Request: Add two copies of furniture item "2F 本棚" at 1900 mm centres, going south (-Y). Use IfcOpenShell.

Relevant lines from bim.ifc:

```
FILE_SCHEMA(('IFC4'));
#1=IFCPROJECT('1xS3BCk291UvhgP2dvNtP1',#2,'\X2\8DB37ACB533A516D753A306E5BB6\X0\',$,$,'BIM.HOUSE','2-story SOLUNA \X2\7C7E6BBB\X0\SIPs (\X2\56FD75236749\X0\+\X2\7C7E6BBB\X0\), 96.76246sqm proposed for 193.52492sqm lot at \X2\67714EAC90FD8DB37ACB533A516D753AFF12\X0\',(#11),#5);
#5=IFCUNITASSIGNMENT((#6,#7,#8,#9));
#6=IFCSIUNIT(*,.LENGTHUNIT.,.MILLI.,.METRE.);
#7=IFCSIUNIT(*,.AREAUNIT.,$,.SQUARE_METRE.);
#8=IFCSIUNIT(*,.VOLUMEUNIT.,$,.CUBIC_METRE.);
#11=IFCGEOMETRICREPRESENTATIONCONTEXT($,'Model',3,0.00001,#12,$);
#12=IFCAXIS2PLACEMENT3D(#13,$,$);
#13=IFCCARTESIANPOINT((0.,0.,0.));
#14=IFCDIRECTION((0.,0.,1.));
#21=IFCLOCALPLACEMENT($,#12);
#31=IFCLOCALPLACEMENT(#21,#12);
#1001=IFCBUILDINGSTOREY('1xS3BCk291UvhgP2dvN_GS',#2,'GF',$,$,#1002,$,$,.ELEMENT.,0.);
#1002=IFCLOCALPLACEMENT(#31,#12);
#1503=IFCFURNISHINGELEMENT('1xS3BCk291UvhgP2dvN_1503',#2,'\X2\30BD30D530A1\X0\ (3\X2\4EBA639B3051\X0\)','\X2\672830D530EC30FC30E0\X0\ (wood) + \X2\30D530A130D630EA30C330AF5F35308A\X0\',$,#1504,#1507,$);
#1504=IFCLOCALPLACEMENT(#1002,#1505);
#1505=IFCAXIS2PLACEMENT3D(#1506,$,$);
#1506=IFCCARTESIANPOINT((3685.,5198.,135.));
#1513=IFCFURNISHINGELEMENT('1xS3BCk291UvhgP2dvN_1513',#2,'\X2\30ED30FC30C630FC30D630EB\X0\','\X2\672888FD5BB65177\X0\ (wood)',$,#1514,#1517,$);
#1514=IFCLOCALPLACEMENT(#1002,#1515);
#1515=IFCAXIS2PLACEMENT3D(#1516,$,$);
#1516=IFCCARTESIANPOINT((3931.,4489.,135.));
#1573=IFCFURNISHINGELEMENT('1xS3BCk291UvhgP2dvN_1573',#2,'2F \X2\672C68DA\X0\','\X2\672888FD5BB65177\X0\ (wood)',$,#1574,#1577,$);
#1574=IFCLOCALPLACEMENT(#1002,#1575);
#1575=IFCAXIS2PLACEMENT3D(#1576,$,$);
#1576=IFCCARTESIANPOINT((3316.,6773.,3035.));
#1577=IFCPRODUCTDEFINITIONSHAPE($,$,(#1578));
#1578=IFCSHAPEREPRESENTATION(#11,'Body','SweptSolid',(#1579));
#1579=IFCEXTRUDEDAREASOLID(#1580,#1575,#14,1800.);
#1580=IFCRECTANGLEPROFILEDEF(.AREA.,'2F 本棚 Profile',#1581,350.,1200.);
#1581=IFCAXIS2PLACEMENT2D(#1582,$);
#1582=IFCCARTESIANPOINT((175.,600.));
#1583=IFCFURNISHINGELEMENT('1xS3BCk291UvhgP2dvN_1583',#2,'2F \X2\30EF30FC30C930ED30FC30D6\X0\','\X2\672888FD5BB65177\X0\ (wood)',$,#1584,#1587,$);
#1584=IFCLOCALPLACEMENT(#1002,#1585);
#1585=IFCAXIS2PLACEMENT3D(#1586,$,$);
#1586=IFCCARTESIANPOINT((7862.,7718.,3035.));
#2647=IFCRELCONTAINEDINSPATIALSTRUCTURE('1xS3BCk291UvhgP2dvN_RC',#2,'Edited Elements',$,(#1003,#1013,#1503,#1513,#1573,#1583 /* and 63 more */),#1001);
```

```python
import numpy as np
import ifcopenshell
import ifcopenshell.api.geometry
import ifcopenshell.api.root
import ifcopenshell.util.element
import ifcopenshell.util.placement

model = ifcopenshell.open("bim.ifc")


def reuse_history(source, copy):
    """copy_class also copies each property set's owner history, people and application; keep the originals."""
    for rel in copy.IsDefinedBy:
        if rel.is_a("IfcRelDefinesByProperties") and (history := rel.RelatingPropertyDefinition.OwnerHistory):
            rel.RelatingPropertyDefinition.OwnerHistory = source.OwnerHistory
            ifcopenshell.util.element.remove_deep2(model, history)


source = model.by_guid("1xS3BCk291UvhgP2dvN_1573")
base = ifcopenshell.util.placement.get_local_placement(source.ObjectPlacement)
step = np.array([0.0, -1.0, 0.0]) * 1900.0

for i in range(1, 3):
    copy = ifcopenshell.api.root.copy_class(model, product=source)
    copy.Representation = ifcopenshell.util.element.copy_deep(
        model, source.Representation, exclude=["IfcGeometricRepresentationContext", "IfcRepresentationMap"]
    )
    reuse_history(source, copy)
    matrix = base.copy()
    matrix[:3, 3] += i * step
    print("added at", matrix[:3, 3].round(3) + 0.0)
    ifcopenshell.api.geometry.edit_object_placement(model, product=copy, matrix=matrix, is_si=False)

model.write("bim_v2.ifc")
```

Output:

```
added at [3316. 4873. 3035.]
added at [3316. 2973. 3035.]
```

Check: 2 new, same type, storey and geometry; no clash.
